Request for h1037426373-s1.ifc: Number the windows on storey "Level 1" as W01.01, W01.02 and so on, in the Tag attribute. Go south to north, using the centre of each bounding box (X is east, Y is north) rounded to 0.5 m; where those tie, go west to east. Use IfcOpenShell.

First a look at what the model holds.

```python
import ifcopenshell
import ifcopenshell.util.element
import ifcopenshell.util.placement

model = ifcopenshell.open("h1037426373-s1.ifc")
print(model.schema)
storey = next(s for s in model.by_type("IfcBuildingStorey") if s.Name == "Level 1")
windows = [e for e in ifcopenshell.util.element.get_decomposition(storey) if e.is_a("IfcWindow")]
for e in sorted(windows, key=lambda e: e.id()):
    origin = ifcopenshell.util.placement.get_local_placement(e.ObjectPlacement)[:3, 3]
    print(e.id(), e.Tag, e.Name, origin.round(2) + 0.0, sep=" | ")
```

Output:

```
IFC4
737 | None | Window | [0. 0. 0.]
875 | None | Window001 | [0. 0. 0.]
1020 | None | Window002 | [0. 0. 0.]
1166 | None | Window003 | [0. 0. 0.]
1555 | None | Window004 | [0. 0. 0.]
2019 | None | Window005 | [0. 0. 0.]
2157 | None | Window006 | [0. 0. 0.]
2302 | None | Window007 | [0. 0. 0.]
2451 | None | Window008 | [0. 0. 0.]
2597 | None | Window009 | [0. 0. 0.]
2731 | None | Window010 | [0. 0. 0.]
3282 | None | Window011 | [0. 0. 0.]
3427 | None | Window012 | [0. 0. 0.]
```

```python
import ifcopenshell
import ifcopenshell.geom
import ifcopenshell.util.element
import ifcopenshell.util.shape

model = ifcopenshell.open("h1037426373-s1.ifc")
settings = ifcopenshell.geom.settings()
settings.set("use-world-coords", True)


def centre(element):
    shape = ifcopenshell.geom.create_shape(settings, element)
    return ifcopenshell.util.shape.get_bbox_centroid(shape.geometry)


storey = next(s for s in model.by_type("IfcBuildingStorey") if s.Name == "Level 1")
windows = [e for e in ifcopenshell.util.element.get_decomposition(storey) if e.is_a("IfcWindow")]

# Insertion points can sit at a corner or the storey origin, so sort by the geometry (in metres).
centres = {e: centre(e) for e in windows}
windows.sort(key=lambda e: (round(centres[e][1] / 0.5), centres[e][0]))

for i, e in enumerate(windows, start=1):
    number = f"W01.{i:02d}"
    e.Tag = number
    print(e.id(), number)

model.write("h1037426373-s1_updated.ifc")
```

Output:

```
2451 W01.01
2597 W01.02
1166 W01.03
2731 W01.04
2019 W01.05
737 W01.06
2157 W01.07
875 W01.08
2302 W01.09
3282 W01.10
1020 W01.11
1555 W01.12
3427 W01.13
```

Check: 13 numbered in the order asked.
